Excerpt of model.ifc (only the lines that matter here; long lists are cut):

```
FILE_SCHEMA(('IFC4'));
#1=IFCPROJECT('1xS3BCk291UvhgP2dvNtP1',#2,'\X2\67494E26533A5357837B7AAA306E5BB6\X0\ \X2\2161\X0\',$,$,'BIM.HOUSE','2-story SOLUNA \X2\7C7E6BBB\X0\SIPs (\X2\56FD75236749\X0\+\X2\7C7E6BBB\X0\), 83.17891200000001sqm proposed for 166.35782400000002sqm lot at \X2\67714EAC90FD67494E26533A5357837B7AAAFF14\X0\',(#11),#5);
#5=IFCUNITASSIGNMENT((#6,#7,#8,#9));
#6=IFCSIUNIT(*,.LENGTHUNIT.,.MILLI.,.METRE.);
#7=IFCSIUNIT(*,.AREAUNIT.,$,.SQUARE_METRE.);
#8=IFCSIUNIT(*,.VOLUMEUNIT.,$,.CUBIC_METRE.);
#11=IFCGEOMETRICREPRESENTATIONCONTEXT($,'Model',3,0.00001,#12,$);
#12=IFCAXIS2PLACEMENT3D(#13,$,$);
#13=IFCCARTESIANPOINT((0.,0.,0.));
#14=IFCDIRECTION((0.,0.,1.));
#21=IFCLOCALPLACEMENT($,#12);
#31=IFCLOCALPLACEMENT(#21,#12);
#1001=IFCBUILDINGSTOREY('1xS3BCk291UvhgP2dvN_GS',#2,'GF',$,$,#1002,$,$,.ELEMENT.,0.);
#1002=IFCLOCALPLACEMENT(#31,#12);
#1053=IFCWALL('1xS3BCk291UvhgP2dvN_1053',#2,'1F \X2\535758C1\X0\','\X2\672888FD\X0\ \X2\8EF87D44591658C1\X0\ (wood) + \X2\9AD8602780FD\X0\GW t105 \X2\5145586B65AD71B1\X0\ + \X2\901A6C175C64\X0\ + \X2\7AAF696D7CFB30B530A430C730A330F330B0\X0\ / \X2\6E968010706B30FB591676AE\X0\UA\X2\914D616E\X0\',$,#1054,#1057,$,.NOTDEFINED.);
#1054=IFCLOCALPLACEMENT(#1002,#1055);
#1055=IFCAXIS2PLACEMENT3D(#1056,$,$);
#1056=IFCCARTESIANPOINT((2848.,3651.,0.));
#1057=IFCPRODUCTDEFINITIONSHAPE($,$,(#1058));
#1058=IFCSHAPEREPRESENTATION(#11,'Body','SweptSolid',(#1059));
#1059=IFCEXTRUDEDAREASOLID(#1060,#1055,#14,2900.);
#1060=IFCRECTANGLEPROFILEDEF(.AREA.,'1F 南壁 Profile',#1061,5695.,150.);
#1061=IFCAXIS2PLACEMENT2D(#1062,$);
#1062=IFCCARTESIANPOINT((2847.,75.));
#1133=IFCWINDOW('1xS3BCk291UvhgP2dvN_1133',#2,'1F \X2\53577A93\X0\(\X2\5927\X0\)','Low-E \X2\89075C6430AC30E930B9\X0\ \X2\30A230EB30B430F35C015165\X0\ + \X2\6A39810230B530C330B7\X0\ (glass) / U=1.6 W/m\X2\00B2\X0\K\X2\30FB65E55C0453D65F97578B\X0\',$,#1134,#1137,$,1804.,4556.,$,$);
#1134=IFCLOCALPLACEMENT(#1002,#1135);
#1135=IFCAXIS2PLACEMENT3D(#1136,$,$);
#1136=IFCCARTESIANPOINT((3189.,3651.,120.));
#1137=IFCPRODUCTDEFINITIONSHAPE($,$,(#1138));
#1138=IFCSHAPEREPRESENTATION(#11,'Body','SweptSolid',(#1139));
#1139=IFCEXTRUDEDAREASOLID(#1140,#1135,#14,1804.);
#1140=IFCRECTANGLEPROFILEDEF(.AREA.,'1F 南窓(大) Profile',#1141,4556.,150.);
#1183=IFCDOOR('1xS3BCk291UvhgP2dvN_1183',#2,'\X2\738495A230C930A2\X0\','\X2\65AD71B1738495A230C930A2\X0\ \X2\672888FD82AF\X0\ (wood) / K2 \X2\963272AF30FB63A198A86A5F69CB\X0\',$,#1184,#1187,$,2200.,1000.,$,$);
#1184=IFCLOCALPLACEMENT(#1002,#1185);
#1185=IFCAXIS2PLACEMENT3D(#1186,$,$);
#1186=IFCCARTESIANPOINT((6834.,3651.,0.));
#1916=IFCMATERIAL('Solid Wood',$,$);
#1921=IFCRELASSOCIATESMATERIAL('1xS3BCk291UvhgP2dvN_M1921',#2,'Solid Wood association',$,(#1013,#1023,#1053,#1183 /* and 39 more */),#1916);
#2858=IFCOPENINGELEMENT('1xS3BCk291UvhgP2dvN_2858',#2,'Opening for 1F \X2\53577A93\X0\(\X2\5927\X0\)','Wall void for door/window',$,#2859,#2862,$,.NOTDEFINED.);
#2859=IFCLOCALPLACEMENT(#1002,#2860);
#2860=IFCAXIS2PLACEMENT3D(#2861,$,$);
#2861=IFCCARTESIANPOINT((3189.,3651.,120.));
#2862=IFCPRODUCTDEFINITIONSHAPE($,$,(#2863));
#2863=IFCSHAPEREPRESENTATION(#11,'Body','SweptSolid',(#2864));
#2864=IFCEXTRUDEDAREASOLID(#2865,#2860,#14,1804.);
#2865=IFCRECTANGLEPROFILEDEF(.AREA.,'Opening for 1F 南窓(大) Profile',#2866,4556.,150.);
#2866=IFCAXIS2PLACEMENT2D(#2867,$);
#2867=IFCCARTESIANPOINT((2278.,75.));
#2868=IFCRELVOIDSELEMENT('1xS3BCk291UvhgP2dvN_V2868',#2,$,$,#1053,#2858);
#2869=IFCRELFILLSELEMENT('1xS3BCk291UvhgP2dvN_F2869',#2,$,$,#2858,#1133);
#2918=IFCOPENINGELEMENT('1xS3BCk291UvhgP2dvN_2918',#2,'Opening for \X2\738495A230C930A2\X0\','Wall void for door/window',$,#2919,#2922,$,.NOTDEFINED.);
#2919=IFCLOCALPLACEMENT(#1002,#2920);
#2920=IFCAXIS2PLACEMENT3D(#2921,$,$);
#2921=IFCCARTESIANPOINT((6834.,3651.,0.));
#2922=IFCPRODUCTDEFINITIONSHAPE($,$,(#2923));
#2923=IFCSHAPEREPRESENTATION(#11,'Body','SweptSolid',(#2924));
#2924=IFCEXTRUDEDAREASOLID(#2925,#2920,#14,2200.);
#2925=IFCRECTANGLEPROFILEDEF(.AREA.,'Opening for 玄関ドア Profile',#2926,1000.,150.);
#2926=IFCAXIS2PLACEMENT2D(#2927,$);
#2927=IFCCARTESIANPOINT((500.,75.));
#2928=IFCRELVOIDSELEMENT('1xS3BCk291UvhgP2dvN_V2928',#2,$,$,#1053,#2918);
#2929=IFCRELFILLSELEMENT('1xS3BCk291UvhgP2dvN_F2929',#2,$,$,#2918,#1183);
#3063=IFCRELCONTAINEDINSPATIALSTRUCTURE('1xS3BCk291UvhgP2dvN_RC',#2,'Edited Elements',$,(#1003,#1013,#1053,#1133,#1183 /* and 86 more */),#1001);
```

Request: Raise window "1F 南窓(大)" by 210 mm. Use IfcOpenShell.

```python
import numpy as np
import ifcopenshell
import ifcopenshell.api.geometry
import ifcopenshell.util.placement
import ifcopenshell.util.unit

model = ifcopenshell.open("model.ifc")
unit_scale = ifcopenshell.util.unit.calculate_unit_scale(model)

window = model.by_guid("1xS3BCk291UvhgP2dvN_1133")
opening = window.FillsVoids[0].RelatingOpeningElement
dz = 0.21 / unit_scale

shift = np.array([0.0, 0.0, dz])
# The window is not placed relative to its opening, so move both.
for product in (opening, window):
    matrix = ifcopenshell.util.placement.get_local_placement(product.ObjectPlacement)
    matrix[:3, 3] += shift
    ifcopenshell.api.geometry.edit_object_placement(model, product=product, matrix=matrix, is_si=False)

print(f"moved by {dz * unit_scale:+.3f} m")

model.write("model-out.ifc")
```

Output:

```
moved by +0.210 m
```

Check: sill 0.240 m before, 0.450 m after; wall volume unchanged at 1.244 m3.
